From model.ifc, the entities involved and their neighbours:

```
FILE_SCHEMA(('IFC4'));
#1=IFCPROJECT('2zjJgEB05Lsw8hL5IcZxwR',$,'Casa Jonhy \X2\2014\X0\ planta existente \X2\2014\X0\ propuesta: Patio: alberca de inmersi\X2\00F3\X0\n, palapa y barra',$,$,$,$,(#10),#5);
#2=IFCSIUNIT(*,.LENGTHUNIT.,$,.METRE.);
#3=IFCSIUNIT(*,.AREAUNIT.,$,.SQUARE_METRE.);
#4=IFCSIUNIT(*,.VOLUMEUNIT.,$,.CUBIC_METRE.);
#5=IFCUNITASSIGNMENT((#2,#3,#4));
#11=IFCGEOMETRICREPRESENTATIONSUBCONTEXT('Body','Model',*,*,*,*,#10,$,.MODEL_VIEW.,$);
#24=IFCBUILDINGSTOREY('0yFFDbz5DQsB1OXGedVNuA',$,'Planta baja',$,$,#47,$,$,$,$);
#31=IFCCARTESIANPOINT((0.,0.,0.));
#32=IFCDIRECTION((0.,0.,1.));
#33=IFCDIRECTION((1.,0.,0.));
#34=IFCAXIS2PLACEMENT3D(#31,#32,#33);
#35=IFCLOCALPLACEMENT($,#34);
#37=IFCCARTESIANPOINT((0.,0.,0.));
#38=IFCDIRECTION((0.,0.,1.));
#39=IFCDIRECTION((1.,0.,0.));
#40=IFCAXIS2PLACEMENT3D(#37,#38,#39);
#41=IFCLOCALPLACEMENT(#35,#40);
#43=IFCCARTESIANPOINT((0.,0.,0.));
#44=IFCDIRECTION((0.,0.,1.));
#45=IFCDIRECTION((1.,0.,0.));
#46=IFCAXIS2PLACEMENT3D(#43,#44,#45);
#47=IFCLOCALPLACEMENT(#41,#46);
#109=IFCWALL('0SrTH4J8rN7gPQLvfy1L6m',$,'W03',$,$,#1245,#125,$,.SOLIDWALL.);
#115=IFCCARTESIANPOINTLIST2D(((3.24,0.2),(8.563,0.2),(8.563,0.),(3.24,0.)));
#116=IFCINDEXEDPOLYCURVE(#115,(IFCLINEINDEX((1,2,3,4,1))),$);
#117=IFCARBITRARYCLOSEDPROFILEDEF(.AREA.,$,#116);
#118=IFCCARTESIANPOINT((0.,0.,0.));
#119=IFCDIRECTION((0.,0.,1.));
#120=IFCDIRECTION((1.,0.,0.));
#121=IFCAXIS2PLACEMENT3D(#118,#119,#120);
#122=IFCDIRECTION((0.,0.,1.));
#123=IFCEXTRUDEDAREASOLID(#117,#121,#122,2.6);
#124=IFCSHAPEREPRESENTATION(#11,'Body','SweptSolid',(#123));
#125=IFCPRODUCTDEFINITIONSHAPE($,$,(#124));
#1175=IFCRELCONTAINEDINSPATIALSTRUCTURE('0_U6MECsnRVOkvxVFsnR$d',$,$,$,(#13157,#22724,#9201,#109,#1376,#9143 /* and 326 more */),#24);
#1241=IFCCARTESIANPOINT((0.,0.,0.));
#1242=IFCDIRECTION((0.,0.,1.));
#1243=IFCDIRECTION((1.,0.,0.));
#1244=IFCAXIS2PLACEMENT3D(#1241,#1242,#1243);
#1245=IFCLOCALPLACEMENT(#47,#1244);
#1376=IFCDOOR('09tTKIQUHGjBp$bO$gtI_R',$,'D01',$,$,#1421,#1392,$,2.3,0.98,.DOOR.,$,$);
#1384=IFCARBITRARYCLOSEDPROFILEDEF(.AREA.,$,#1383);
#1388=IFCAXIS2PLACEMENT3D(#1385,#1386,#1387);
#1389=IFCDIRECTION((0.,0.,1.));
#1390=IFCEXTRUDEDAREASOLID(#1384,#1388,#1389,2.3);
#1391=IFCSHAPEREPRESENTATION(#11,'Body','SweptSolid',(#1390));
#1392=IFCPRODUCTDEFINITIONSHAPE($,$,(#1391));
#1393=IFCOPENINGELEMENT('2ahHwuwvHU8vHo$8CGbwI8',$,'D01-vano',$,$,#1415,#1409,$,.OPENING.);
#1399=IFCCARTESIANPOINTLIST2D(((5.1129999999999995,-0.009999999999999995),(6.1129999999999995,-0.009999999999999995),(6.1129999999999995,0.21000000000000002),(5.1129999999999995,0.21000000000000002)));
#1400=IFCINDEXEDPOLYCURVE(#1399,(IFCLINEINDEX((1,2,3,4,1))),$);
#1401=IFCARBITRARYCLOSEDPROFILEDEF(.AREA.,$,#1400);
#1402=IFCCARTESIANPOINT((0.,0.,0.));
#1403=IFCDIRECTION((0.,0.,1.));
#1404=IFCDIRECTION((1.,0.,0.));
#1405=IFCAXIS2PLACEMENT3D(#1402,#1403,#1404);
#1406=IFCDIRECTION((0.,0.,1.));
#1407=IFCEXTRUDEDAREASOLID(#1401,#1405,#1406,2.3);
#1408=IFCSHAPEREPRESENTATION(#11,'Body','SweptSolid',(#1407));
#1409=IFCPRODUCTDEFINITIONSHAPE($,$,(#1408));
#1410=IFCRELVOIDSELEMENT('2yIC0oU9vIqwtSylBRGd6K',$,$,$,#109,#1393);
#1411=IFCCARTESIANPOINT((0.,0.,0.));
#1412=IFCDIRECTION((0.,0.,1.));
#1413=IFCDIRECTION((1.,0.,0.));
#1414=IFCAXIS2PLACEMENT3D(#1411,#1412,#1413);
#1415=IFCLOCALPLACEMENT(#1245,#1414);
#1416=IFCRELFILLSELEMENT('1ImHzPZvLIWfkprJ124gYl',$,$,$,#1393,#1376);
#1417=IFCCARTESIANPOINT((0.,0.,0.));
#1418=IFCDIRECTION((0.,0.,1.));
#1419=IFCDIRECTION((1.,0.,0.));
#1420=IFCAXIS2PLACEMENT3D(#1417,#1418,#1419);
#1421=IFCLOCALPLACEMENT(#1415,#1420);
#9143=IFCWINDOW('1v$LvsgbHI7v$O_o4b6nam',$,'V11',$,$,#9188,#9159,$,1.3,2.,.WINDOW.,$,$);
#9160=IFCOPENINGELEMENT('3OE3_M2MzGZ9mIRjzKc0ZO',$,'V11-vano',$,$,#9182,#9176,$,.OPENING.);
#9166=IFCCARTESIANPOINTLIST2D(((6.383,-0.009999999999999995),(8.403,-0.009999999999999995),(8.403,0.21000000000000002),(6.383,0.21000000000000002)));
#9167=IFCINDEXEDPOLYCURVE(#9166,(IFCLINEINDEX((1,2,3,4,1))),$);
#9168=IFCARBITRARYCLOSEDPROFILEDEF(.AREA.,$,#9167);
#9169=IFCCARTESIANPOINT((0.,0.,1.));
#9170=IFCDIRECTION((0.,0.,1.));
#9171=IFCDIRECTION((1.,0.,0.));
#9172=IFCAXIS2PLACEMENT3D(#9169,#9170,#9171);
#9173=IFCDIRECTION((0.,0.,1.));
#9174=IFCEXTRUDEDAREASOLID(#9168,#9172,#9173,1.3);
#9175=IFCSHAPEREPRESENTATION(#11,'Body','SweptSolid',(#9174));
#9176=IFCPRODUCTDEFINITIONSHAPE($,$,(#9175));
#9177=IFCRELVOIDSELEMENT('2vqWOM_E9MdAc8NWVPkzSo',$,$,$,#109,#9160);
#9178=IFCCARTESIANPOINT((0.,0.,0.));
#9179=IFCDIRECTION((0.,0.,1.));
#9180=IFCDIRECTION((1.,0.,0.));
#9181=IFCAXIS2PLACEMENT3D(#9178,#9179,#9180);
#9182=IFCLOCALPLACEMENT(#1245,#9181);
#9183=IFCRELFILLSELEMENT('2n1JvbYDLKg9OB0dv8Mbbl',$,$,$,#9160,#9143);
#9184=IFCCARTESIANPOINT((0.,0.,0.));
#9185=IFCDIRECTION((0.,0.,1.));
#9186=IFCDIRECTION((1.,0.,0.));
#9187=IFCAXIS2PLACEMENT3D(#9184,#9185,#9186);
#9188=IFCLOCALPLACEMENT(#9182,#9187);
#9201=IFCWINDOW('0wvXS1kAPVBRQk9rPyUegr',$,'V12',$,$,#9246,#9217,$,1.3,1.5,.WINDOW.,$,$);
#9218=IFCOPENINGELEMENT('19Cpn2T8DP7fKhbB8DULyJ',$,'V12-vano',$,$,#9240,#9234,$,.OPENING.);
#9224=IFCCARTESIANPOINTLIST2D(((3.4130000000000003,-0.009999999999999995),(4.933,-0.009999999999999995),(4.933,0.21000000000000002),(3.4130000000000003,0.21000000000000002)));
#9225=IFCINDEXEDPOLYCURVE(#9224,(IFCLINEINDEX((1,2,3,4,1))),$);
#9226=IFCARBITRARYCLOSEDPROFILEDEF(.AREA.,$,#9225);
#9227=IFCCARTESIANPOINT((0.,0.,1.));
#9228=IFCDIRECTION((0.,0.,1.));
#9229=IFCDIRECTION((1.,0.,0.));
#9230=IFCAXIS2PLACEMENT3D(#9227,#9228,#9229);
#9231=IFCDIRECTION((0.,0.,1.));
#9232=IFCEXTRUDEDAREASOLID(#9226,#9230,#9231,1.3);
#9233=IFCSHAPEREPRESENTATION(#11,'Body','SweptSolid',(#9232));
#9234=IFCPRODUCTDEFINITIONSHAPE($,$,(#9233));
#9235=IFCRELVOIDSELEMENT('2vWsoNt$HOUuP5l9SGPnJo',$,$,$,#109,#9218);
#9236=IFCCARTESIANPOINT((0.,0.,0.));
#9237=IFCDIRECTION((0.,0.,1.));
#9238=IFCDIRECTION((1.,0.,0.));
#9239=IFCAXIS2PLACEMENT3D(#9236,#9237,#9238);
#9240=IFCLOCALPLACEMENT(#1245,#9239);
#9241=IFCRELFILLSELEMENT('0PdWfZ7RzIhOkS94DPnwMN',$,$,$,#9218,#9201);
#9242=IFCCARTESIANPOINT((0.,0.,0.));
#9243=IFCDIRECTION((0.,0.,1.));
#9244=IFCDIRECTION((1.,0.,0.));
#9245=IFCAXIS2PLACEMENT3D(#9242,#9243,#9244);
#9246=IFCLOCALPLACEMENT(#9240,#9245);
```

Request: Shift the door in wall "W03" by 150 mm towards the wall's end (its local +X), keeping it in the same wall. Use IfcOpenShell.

```python
import ifcopenshell
import ifcopenshell.api.geometry
import ifcopenshell.util.placement

model = ifcopenshell.open("model.ifc")

door = model.by_id(1376)
opening = door.FillsVoids[0].RelatingOpeningElement
wall = opening.VoidsElements[0].RelatingBuildingElement

wall_matrix = ifcopenshell.util.placement.get_local_placement(wall.ObjectPlacement)
shift = wall_matrix[:3, 0] * 0.15
before = ifcopenshell.util.placement.get_local_placement(door.ObjectPlacement)[:3, 3].copy()

# The door is placed relative to its opening, so it follows when the opening moves.
matrix = ifcopenshell.util.placement.get_local_placement(opening.ObjectPlacement)
matrix[:3, 3] += shift
ifcopenshell.api.geometry.edit_object_placement(
    model, product=opening, matrix=matrix, is_si=False, should_transform_children=True
)

after = ifcopenshell.util.placement.get_local_placement(door.ObjectPlacement)[:3, 3]
print("door moved by", (after - before).round(3) + 0.0)

model.write("model_edited.ifc")
```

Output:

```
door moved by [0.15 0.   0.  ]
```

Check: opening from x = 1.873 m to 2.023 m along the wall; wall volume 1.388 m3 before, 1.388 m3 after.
